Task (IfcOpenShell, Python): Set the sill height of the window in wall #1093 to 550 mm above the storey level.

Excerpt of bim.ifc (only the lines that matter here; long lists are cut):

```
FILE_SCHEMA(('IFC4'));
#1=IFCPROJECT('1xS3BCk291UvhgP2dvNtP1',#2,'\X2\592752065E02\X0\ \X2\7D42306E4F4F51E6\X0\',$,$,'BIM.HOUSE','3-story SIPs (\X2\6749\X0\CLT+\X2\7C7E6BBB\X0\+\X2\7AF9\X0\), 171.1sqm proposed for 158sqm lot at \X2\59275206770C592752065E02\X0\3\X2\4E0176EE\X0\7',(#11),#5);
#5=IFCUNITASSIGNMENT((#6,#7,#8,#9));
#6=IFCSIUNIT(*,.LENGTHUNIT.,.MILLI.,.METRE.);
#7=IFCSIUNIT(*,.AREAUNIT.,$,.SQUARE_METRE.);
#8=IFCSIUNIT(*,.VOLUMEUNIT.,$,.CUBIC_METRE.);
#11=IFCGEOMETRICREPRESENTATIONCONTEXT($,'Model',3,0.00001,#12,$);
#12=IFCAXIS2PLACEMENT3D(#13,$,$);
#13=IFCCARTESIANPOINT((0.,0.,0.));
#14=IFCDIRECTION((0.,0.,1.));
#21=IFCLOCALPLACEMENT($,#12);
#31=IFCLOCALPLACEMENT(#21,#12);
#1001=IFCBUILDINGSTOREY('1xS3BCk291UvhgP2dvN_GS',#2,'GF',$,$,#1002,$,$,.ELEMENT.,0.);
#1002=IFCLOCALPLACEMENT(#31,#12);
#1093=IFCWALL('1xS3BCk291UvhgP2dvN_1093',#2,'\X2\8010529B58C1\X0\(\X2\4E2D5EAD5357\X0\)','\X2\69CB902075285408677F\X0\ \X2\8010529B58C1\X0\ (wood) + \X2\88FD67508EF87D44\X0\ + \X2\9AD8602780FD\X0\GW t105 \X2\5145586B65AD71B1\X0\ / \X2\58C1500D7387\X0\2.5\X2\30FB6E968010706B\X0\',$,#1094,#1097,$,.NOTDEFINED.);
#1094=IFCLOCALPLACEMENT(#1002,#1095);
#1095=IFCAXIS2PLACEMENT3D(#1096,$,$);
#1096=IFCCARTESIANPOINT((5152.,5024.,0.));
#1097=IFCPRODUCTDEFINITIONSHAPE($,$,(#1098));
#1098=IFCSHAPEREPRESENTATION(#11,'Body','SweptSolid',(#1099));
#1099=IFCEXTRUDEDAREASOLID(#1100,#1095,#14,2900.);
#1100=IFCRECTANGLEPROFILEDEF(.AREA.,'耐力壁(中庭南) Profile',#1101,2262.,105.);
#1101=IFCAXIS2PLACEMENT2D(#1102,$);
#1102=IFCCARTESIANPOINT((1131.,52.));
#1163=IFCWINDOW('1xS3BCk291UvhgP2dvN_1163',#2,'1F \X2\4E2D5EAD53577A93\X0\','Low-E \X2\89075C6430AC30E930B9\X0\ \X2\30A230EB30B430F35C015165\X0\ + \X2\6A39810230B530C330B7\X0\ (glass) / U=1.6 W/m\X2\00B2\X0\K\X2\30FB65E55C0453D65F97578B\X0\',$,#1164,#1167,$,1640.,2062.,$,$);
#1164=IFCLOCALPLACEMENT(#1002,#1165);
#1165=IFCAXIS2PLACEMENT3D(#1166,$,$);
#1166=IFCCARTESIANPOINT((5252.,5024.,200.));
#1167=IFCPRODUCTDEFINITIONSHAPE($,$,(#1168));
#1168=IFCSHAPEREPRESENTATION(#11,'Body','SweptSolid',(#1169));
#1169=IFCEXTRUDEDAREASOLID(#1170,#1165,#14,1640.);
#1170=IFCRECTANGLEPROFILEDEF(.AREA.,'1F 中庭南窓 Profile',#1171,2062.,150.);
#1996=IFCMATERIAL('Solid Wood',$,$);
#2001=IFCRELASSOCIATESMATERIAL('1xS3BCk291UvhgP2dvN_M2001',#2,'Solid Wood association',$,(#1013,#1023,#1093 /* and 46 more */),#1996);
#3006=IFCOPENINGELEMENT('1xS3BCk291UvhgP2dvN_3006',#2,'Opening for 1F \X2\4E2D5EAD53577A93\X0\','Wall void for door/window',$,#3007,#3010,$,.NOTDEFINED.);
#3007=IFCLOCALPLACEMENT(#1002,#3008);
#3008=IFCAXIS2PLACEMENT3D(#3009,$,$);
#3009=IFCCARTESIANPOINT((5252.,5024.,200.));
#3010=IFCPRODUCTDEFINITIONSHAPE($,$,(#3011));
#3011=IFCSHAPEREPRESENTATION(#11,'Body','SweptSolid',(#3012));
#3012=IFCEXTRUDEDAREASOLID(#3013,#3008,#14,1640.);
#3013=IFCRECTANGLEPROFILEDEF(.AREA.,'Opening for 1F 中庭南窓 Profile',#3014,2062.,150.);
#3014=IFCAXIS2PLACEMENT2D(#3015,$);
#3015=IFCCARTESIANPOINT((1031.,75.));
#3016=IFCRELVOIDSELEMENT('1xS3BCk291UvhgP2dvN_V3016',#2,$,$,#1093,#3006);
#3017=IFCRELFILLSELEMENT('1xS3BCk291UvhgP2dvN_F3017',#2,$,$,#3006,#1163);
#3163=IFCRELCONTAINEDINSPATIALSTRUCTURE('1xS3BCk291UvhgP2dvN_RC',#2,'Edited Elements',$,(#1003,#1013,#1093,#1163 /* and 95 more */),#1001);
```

```python
import numpy as np
import ifcopenshell
import ifcopenshell.api.geometry
import ifcopenshell.geom
import ifcopenshell.util.element
import ifcopenshell.util.placement
import ifcopenshell.util.shape
import ifcopenshell.util.unit

model = ifcopenshell.open("bim.ifc")
unit_scale = ifcopenshell.util.unit.calculate_unit_scale(model)

window = model.by_id(1163)
opening = window.FillsVoids[0].RelatingOpeningElement
storey = ifcopenshell.util.element.get_container(window, ifc_class="IfcBuildingStorey")
level = ifcopenshell.util.placement.get_local_placement(storey.ObjectPlacement)[2, 3]

# The opening's origin need not be at the sill, so measure its lowest point.
shape = ifcopenshell.geom.create_shape(ifcopenshell.geom.settings(), opening)
bottom = ifcopenshell.util.shape.get_shape_bottom_elevation(shape, shape.geometry) / unit_scale
dz = level + 0.55 / unit_scale - bottom

shift = np.array([0.0, 0.0, dz])
# The window is not placed relative to its opening, so move both.
for product in (opening, window):
    matrix = ifcopenshell.util.placement.get_local_placement(product.ObjectPlacement)
    matrix[:3, 3] += shift
    ifcopenshell.api.geometry.edit_object_placement(model, product=product, matrix=matrix, is_si=False)

print(f"moved by {dz * unit_scale:+.3f} m")

model.write("bim-out.ifc")
```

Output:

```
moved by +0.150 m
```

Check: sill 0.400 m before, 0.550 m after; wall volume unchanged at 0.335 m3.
